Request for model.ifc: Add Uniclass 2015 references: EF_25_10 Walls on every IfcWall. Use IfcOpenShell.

First a look at what the model holds.

```python
import ifcopenshell

model = ifcopenshell.open("model.ifc")
print(model.schema)
print("classifications:", [c.Name for c in model.by_type("IfcClassification")])
for ifc_class in ("IfcDoor", "IfcRoof", "IfcStair", "IfcWall", "IfcWindow"):
    print(ifc_class, len(model.by_type(ifc_class)))
```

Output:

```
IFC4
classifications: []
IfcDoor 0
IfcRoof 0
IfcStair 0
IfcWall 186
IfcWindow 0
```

```python
import ifcopenshell
import ifcopenshell.api.classification

model = ifcopenshell.open("model.ifc")

system = ifcopenshell.api.classification.add_classification(model, classification="Uniclass 2015")

codes = {
    "IfcWall": ("EF_25_10", "Walls"),
}
for ifc_class, (code, name) in codes.items():
    products = model.by_type(ifc_class)
    ifcopenshell.api.classification.add_reference(
        model, products=products, classification=system, identification=code, name=name
    )
    print(code, len(products))

model.write("model_edited.ifc")
```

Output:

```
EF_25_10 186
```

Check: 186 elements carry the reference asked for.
